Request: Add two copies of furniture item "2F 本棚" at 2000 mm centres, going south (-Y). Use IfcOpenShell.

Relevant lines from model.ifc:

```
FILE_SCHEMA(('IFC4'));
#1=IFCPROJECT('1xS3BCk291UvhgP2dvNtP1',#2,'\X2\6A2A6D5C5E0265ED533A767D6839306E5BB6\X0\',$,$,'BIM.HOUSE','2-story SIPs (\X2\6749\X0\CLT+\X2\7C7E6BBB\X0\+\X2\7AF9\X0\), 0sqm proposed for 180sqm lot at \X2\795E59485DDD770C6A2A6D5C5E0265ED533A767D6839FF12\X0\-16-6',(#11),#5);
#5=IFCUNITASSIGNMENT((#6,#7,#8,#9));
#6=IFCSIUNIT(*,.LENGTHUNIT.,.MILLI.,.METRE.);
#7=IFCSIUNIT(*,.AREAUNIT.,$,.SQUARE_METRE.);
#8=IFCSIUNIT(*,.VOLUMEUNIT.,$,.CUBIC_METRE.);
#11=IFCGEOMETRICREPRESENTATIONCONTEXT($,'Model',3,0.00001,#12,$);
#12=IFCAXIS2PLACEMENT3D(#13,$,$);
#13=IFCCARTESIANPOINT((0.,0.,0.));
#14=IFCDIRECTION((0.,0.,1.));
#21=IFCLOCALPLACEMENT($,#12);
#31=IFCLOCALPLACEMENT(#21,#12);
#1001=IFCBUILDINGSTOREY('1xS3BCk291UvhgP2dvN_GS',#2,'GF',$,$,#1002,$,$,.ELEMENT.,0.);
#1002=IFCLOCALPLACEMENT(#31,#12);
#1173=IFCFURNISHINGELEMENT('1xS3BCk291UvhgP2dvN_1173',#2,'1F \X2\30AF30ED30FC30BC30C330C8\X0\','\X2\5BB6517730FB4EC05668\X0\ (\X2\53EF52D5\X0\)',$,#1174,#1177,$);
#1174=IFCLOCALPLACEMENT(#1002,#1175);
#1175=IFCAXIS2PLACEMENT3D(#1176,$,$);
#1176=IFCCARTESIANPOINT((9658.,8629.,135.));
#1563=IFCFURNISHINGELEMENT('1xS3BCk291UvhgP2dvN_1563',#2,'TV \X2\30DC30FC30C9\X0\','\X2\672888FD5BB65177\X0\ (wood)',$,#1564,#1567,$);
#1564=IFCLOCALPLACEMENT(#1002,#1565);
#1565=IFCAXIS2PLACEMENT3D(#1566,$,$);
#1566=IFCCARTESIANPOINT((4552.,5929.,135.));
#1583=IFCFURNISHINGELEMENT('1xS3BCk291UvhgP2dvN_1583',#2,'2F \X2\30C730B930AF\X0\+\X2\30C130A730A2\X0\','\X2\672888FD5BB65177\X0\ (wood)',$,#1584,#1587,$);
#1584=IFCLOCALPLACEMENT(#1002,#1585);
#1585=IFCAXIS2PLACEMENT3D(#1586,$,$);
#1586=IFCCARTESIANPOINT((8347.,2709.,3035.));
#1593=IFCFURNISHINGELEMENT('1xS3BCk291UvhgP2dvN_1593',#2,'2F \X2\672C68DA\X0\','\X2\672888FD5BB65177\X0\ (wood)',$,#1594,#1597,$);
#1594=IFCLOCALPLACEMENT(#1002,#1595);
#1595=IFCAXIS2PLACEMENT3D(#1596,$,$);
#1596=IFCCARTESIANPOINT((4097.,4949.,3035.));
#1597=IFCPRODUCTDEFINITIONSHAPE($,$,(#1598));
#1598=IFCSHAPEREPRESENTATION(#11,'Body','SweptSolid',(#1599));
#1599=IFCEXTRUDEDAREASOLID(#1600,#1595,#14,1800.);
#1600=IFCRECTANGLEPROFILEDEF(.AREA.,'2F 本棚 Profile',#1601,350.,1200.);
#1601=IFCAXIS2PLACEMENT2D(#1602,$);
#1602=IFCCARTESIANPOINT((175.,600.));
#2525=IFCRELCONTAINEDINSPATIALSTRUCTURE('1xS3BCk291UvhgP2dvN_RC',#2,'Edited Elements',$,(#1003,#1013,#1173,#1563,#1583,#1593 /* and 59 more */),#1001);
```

```python
import numpy as np
import ifcopenshell
import ifcopenshell.api.geometry
import ifcopenshell.api.root
import ifcopenshell.util.element
import ifcopenshell.util.placement
import ifcopenshell.util.unit

model = ifcopenshell.open("model.ifc")
unit_scale = ifcopenshell.util.unit.calculate_unit_scale(model)


def reuse_history(source, copy):
    """copy_class also copies each property set's owner history, people and application; keep the originals."""
    for rel in copy.IsDefinedBy:
        if rel.is_a("IfcRelDefinesByProperties") and (history := rel.RelatingPropertyDefinition.OwnerHistory):
            rel.RelatingPropertyDefinition.OwnerHistory = source.OwnerHistory
            ifcopenshell.util.element.remove_deep2(model, history)


source = model.by_id(1593)
base = ifcopenshell.util.placement.get_local_placement(source.ObjectPlacement)
step = np.array([0.0, -1.0, 0.0]) * 2 / unit_scale

for i in range(1, 3):
    copy = ifcopenshell.api.root.copy_class(model, product=source)
    copy.Representation = ifcopenshell.util.element.copy_deep(
        model, source.Representation, exclude=["IfcGeometricRepresentationContext", "IfcRepresentationMap"]
    )
    reuse_history(source, copy)
    matrix = base.copy()
    matrix[:3, 3] += i * step
    print("added at", matrix[:3, 3].round(3) + 0.0)
    ifcopenshell.api.geometry.edit_object_placement(model, product=copy, matrix=matrix, is_si=False)

model.write("model-out.ifc")
```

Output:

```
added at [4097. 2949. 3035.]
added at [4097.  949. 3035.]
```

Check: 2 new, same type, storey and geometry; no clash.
